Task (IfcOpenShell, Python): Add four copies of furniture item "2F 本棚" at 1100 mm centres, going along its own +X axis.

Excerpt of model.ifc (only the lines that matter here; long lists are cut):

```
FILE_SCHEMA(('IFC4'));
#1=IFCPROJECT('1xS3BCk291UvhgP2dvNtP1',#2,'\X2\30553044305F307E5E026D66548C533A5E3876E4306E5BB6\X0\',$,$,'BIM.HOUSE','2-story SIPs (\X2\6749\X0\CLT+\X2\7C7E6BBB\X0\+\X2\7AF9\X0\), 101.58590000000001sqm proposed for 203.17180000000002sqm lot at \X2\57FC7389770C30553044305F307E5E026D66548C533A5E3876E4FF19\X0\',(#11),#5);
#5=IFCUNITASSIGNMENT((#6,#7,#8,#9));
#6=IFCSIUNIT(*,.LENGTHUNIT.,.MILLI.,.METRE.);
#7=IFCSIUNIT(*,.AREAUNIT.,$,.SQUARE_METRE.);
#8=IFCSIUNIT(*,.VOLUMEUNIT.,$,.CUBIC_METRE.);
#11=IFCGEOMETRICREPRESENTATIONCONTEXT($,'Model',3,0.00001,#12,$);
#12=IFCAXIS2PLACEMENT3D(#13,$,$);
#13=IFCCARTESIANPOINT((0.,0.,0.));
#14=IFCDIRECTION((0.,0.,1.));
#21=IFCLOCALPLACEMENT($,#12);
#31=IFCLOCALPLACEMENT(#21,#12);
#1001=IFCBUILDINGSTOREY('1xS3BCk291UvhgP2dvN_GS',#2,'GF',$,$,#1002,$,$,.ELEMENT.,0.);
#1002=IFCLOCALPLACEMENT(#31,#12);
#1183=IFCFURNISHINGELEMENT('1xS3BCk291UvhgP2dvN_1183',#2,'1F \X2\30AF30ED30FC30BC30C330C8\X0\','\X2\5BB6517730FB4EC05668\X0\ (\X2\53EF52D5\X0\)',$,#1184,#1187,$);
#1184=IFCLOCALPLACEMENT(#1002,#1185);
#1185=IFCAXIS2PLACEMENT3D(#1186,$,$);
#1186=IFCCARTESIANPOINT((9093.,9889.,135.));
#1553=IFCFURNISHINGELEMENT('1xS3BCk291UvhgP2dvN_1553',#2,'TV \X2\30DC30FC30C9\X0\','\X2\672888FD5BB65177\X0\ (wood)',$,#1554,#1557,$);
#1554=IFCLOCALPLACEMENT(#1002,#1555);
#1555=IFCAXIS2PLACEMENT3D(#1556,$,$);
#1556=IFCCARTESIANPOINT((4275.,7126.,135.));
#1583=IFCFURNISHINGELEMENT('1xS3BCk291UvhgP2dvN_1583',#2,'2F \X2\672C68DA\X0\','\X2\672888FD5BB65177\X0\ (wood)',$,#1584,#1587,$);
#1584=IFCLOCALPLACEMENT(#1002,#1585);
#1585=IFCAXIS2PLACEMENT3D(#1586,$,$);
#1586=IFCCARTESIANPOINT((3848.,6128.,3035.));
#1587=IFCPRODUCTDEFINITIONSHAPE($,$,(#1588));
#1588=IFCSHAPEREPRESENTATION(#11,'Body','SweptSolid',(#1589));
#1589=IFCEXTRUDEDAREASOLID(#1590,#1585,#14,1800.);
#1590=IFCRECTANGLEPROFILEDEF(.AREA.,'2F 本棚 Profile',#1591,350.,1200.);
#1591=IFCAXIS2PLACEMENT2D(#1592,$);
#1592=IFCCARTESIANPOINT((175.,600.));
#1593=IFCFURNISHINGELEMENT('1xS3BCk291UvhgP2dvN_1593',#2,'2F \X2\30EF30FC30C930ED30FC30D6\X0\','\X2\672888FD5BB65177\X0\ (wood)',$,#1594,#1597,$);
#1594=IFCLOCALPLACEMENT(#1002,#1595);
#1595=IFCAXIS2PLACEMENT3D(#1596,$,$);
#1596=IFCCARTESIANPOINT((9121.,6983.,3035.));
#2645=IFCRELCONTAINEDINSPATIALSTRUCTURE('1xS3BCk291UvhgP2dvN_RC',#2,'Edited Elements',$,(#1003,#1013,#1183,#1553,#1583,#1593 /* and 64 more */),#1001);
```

```python
import ifcopenshell
import ifcopenshell.api.geometry
import ifcopenshell.api.root
import ifcopenshell.util.element
import ifcopenshell.util.placement
import ifcopenshell.util.unit

model = ifcopenshell.open("model.ifc")
unit_scale = ifcopenshell.util.unit.calculate_unit_scale(model)


def reuse_history(source, copy):
    """copy_class also copies each property set's owner history, people and application; keep the originals."""
    for rel in copy.IsDefinedBy:
        if rel.is_a("IfcRelDefinesByProperties") and (history := rel.RelatingPropertyDefinition.OwnerHistory):
            rel.RelatingPropertyDefinition.OwnerHistory = source.OwnerHistory
            ifcopenshell.util.element.remove_deep2(model, history)


source = model.by_id(1583)
base = ifcopenshell.util.placement.get_local_placement(source.ObjectPlacement)
step = base[:3, 0] * 1.1 / unit_scale

for i in range(1, 5):
    copy = ifcopenshell.api.root.copy_class(model, product=source)
    copy.Representation = ifcopenshell.util.element.copy_deep(
        model, source.Representation, exclude=["IfcGeometricRepresentationContext", "IfcRepresentationMap"]
    )
    reuse_history(source, copy)
    matrix = base.copy()
    matrix[:3, 3] += i * step
    print("added at", matrix[:3, 3].round(3) + 0.0)
    ifcopenshell.api.geometry.edit_object_placement(model, product=copy, matrix=matrix, is_si=False)

model.write("model-out.ifc")
```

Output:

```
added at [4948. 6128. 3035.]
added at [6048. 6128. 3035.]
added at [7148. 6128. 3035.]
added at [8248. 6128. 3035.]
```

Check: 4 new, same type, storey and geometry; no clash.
